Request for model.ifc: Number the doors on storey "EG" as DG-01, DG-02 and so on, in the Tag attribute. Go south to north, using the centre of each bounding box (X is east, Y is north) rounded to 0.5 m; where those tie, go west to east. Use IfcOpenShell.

First a look at what the model holds.

```python
import ifcopenshell
import ifcopenshell.util.element
import ifcopenshell.util.placement

model = ifcopenshell.open("model.ifc")
print(model.schema)
storey = next(s for s in model.by_type("IfcBuildingStorey") if s.Name == "EG")
doors = [e for e in ifcopenshell.util.element.get_decomposition(storey) if e.is_a("IfcDoor")]
for e in sorted(doors, key=lambda e: e.id()):
    origin = ifcopenshell.util.placement.get_local_placement(e.ObjectPlacement)[:3, 3]
    print(e.id(), e.Tag, e.Name, origin.round(2) + 0.0, sep=" | ")
```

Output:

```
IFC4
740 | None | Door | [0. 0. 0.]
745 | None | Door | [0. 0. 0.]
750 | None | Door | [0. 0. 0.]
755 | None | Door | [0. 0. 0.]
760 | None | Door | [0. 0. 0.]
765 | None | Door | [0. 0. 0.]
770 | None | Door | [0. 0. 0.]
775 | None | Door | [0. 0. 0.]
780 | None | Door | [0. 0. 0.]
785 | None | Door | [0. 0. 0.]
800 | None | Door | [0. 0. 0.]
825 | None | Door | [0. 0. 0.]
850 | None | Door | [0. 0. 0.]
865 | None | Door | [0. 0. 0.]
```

```python
import ifcopenshell
import ifcopenshell.geom
import ifcopenshell.util.element
import ifcopenshell.util.shape

model = ifcopenshell.open("model.ifc")
settings = ifcopenshell.geom.settings()
settings.set("use-world-coords", True)


def centre(element):
    shape = ifcopenshell.geom.create_shape(settings, element)
    return ifcopenshell.util.shape.get_bbox_centroid(shape.geometry)


storey = next(s for s in model.by_type("IfcBuildingStorey") if s.Name == "EG")
doors = [e for e in ifcopenshell.util.element.get_decomposition(storey) if e.is_a("IfcDoor")]

# Insertion points can sit at a corner or the storey origin, so sort by the geometry (in metres).
centres = {e: centre(e) for e in doors}
doors.sort(key=lambda e: (round(centres[e][1] / 0.5), centres[e][0]))

for i, e in enumerate(doors, start=1):
    number = f"DG-{i:02d}"
    e.Tag = number
    print(e.id(), number)

model.write("model_v2.ifc")
```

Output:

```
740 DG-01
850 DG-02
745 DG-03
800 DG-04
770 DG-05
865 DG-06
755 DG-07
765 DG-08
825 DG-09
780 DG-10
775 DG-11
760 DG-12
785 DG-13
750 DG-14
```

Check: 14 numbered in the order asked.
